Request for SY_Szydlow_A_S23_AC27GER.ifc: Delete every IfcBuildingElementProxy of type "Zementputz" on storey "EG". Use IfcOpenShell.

First a look at what the model holds.

```python
import ifcopenshell
import ifcopenshell.util.element

model = ifcopenshell.open("SY_Szydlow_A_S23_AC27GER.ifc")
print(model.schema)
storey = next(s for s in model.by_type("IfcBuildingStorey") if s.Name == "EG")
proxies = [e for e in ifcopenshell.util.element.get_decomposition(storey) if e.is_a("IfcBuildingElementProxy")]
seen = {}
for e in proxies:
    element_type = ifcopenshell.util.element.get_type(e)
    name = element_type.Name if element_type not in (None, e) else None
    seen[name] = seen.get(name, 0) + 1
for name, count in sorted(seen.items(), key=str):
    print(count, "x", name)
```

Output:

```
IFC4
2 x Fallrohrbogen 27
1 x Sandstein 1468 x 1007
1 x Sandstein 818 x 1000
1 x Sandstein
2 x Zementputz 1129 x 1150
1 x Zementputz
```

```python
import ifcopenshell
import ifcopenshell.api.root
import ifcopenshell.util.element

model = ifcopenshell.open("SY_Szydlow_A_S23_AC27GER.ifc")

storey = next(s for s in model.by_type("IfcBuildingStorey") if s.Name == "EG")
proxies = [e for e in ifcopenshell.util.element.get_decomposition(storey) if e.is_a("IfcBuildingElementProxy")]
targets = [e for e in proxies if (t := ifcopenshell.util.element.get_type(e)) not in (None, e) and t.Name == "Zementputz"]

for e in targets:
    ifcopenshell.api.root.remove_product(model, product=e)
print(len(targets), "removed")

model.write("SY_Szydlow_A_S23_AC27GER_edited.ifc")
```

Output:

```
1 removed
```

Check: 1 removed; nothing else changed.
